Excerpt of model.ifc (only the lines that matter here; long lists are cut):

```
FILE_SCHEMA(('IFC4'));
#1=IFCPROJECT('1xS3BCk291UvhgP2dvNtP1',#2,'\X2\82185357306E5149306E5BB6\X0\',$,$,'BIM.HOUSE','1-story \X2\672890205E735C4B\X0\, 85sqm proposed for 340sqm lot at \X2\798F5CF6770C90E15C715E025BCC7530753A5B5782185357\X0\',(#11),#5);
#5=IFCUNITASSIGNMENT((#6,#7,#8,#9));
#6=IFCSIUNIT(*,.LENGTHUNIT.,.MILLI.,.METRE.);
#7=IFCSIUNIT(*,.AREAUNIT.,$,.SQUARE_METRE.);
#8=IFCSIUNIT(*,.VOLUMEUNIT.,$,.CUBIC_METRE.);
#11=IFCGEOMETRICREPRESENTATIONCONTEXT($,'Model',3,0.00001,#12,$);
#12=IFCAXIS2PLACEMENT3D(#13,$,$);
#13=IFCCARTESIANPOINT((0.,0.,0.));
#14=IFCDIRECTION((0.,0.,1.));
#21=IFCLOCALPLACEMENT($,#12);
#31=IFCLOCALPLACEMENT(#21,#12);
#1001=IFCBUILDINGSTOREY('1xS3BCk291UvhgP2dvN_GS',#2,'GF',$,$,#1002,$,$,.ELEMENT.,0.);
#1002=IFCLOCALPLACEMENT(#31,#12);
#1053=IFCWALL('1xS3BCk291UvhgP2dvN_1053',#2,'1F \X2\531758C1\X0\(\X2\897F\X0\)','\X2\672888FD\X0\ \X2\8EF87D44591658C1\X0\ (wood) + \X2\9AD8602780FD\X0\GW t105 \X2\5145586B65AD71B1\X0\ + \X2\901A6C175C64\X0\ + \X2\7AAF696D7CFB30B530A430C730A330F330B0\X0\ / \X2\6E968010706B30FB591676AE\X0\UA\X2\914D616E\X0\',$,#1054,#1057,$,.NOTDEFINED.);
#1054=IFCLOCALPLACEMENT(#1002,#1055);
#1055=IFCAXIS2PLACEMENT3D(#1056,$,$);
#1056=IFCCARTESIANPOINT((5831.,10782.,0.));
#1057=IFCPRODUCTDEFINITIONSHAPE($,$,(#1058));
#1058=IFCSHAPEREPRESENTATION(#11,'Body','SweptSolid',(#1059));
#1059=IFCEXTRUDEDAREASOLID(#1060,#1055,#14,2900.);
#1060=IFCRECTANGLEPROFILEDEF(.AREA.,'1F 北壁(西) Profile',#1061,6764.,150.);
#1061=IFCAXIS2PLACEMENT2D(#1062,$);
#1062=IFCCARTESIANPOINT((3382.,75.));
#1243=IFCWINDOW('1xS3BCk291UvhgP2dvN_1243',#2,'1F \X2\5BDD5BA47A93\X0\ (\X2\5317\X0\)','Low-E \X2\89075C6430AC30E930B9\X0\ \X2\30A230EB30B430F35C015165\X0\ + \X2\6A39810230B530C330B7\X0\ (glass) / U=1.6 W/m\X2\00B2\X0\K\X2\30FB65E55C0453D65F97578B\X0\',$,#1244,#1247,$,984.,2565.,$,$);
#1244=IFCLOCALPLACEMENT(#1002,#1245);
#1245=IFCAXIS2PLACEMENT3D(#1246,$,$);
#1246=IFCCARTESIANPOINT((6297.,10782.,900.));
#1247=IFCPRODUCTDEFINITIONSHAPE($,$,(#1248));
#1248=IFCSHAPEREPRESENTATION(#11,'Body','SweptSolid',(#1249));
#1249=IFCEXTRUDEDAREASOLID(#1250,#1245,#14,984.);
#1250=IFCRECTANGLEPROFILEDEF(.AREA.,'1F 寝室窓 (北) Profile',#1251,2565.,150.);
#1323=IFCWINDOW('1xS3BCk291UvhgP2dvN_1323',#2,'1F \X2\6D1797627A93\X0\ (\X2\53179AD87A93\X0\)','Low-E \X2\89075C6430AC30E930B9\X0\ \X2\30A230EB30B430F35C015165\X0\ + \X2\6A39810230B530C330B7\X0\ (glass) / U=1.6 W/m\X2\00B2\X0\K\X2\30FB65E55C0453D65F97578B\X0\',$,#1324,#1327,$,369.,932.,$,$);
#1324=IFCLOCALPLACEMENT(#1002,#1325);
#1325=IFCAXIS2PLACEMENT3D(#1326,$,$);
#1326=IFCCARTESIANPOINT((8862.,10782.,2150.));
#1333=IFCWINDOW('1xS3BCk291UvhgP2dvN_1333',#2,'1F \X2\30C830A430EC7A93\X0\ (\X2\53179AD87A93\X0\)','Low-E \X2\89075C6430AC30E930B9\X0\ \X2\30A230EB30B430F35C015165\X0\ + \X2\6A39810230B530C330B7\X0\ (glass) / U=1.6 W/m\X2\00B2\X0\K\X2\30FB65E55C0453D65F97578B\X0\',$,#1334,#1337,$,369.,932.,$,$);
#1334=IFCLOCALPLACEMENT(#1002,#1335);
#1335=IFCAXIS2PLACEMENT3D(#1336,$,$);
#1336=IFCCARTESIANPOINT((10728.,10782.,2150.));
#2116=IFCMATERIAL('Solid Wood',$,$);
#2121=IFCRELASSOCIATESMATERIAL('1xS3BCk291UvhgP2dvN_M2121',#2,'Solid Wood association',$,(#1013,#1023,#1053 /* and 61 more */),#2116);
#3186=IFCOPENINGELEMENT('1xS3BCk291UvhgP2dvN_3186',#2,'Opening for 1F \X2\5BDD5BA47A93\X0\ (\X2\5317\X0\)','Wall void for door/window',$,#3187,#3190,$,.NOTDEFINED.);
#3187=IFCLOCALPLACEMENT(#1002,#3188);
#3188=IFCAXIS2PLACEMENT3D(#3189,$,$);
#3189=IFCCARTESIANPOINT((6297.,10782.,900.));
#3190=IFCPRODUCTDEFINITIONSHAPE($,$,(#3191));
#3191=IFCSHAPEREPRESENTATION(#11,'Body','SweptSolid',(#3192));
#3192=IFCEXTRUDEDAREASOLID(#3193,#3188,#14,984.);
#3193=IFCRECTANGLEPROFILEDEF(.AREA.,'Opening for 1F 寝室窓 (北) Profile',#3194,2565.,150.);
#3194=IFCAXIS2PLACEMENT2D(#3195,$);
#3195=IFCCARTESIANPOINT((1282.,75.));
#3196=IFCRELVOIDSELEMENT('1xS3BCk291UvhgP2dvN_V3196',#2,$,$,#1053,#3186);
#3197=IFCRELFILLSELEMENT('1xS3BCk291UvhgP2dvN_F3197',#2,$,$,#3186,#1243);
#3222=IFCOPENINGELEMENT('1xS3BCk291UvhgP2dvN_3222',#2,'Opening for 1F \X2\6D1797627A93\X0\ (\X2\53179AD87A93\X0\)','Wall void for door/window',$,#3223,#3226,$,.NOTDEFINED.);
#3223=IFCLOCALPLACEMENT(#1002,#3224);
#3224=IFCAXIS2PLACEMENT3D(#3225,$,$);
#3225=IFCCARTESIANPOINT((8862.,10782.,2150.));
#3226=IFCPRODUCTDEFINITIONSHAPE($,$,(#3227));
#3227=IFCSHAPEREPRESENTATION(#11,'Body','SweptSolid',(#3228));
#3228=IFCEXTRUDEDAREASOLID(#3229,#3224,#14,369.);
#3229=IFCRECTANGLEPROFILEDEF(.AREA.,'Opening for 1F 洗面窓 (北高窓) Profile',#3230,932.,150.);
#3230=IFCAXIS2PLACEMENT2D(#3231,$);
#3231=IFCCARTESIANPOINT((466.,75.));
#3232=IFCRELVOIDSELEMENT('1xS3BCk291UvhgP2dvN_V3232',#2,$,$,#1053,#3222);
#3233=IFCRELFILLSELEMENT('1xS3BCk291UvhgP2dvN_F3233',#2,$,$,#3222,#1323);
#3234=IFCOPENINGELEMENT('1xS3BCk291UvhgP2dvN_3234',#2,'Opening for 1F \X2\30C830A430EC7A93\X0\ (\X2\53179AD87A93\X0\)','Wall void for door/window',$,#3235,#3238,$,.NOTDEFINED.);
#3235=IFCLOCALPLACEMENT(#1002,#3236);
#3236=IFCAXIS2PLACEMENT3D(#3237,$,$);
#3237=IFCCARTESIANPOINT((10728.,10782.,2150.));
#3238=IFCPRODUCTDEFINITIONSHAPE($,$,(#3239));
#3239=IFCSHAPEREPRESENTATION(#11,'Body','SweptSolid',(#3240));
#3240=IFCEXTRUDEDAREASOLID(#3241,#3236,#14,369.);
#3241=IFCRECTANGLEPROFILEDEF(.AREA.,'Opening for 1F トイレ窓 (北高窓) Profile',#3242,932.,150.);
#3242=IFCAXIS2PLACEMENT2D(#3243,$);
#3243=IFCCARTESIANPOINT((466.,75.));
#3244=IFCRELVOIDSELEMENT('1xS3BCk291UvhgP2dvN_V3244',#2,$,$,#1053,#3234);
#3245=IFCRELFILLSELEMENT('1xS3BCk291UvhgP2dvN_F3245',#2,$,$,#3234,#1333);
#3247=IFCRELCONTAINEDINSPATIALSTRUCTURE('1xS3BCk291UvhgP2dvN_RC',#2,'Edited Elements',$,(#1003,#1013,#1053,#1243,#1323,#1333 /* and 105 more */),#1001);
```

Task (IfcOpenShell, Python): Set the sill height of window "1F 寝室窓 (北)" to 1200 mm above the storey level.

```python
import numpy as np
import ifcopenshell
import ifcopenshell.api.geometry
import ifcopenshell.geom
import ifcopenshell.util.element
import ifcopenshell.util.placement
import ifcopenshell.util.shape
import ifcopenshell.util.unit

model = ifcopenshell.open("model.ifc")
unit_scale = ifcopenshell.util.unit.calculate_unit_scale(model)

window = model.by_guid("1xS3BCk291UvhgP2dvN_1243")
opening = window.FillsVoids[0].RelatingOpeningElement
storey = ifcopenshell.util.element.get_container(window, ifc_class="IfcBuildingStorey")
level = ifcopenshell.util.placement.get_local_placement(storey.ObjectPlacement)[2, 3]

# The opening's origin need not be at the sill, so measure its lowest point.
shape = ifcopenshell.geom.create_shape(ifcopenshell.geom.settings(), opening)
bottom = ifcopenshell.util.shape.get_shape_bottom_elevation(shape, shape.geometry) / unit_scale
dz = level + 1.2 / unit_scale - bottom

shift = np.array([0.0, 0.0, dz])
# The window is not placed relative to its opening, so move both.
for product in (opening, window):
    matrix = ifcopenshell.util.placement.get_local_placement(product.ObjectPlacement)
    matrix[:3, 3] += shift
    ifcopenshell.api.geometry.edit_object_placement(model, product=product, matrix=matrix, is_si=False)

print(f"moved by {dz * unit_scale:+.3f} m")

model.write("model_rev.ifc")
```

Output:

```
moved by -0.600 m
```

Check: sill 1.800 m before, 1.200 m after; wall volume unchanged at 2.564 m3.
